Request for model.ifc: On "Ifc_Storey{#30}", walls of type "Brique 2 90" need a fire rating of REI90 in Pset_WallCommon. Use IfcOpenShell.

First a look at what the model holds.

```python
import ifcopenshell
import ifcopenshell.util.element

model = ifcopenshell.open("model.ifc")
print(model.schema)
storey = next(s for s in model.by_type("IfcBuildingStorey") if s.Name == "Ifc_Storey{#30}")
walls = [e for e in ifcopenshell.util.element.get_decomposition(storey) if e.is_a("IfcWall")]
seen = {}
for e in walls:
    element_type = ifcopenshell.util.element.get_type(e)
    key = (element_type.Name if element_type != e and element_type else None, ifcopenshell.util.element.get_pset(e, "Pset_WallCommon", "FireRating"))
    seen[key] = seen.get(key, 0) + 1
for (name, value), count in sorted(seen.items(), key=str):
    print(count, "x", name, "|", value)
```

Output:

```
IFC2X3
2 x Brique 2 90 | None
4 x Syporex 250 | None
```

```python
import ifcopenshell
import ifcopenshell.api.pset
import ifcopenshell.util.element

model = ifcopenshell.open("model.ifc")

storey = next(s for s in model.by_type("IfcBuildingStorey") if s.Name == "Ifc_Storey{#30}")
walls = [e for e in ifcopenshell.util.element.get_decomposition(storey) if e.is_a("IfcWall")]

count = 0
for e in walls:
    element_type = ifcopenshell.util.element.get_type(e)
    if element_type in (None, e) or element_type.Name != "Brique 2 90":
        continue
    # add_pset returns the element's existing set when there is one.
    pset = ifcopenshell.api.pset.add_pset(model, product=e, name="Pset_WallCommon")
    ifcopenshell.api.pset.edit_pset(model, pset=pset, properties={"FireRating": "REI90"})
    count += 1

print(count, "walls updated")

model.write("model_updated.ifc")
```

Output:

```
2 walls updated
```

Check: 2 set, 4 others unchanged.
